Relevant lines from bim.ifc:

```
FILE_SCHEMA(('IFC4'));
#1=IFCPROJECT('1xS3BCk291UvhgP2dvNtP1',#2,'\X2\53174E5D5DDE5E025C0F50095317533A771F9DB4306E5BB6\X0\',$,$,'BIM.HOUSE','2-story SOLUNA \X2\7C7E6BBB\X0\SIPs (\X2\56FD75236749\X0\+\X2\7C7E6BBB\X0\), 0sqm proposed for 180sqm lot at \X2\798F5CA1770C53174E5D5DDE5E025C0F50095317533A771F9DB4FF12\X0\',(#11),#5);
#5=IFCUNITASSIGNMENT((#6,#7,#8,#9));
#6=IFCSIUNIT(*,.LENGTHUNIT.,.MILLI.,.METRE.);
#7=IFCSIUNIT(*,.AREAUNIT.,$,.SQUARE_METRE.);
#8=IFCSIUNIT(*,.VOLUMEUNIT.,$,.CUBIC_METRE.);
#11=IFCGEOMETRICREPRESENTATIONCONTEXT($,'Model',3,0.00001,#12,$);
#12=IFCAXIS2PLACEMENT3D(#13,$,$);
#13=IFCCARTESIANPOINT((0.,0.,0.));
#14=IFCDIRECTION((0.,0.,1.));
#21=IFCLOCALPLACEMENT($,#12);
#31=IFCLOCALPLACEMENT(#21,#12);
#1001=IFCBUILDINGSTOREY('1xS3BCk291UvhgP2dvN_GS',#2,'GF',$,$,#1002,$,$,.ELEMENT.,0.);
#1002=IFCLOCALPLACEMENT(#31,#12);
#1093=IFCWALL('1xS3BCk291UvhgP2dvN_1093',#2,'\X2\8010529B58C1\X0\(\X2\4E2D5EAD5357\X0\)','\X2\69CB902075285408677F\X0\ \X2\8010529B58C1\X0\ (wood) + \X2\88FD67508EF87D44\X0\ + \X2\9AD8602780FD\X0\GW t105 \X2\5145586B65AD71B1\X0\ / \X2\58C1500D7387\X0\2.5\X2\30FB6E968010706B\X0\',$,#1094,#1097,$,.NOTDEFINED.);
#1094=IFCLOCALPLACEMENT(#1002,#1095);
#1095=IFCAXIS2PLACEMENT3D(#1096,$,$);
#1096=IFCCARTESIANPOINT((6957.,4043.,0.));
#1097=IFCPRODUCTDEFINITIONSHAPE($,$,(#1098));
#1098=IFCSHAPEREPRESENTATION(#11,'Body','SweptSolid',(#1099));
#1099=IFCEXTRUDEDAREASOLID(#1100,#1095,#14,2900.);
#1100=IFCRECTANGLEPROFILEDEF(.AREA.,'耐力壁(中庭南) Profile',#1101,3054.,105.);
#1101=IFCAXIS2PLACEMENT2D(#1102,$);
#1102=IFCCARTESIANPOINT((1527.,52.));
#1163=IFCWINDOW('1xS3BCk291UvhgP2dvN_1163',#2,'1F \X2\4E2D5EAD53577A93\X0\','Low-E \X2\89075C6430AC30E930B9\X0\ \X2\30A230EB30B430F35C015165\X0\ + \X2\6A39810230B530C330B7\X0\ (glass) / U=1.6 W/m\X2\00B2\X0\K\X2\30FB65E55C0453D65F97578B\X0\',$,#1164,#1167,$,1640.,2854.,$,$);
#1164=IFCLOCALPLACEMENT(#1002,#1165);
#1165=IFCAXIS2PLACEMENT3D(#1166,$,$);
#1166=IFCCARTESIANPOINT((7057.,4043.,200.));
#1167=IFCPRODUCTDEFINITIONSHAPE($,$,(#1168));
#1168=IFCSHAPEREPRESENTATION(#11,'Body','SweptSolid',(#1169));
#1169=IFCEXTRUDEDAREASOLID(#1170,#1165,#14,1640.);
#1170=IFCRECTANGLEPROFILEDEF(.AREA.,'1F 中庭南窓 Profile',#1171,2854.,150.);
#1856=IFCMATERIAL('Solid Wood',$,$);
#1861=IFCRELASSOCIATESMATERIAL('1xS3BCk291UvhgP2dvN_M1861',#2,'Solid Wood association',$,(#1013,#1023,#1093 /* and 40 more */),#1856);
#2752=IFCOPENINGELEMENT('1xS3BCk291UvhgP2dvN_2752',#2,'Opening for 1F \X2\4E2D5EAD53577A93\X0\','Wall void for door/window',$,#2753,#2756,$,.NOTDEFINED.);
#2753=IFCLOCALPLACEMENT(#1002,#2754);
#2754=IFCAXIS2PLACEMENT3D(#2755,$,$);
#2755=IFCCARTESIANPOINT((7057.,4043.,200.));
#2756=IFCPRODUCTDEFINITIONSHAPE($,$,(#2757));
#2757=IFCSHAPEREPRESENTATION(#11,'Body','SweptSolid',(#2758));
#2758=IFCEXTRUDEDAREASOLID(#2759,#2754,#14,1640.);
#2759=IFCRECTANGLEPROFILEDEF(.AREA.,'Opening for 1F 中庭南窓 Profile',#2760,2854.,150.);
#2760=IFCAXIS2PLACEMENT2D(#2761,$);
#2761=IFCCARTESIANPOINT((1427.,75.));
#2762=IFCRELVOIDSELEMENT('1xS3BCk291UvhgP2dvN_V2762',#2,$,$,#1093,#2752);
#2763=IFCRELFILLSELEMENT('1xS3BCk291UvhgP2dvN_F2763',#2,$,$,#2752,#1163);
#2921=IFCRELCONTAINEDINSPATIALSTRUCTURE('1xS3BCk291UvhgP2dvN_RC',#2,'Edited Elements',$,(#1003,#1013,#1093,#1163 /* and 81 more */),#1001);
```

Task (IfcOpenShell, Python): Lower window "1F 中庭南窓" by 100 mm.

```python
import numpy as np
import ifcopenshell
import ifcopenshell.api.geometry
import ifcopenshell.util.placement
import ifcopenshell.util.unit

model = ifcopenshell.open("bim.ifc")
unit_scale = ifcopenshell.util.unit.calculate_unit_scale(model)

window = model.by_guid("1xS3BCk291UvhgP2dvN_1163")
opening = window.FillsVoids[0].RelatingOpeningElement
dz = -100.0

shift = np.array([0.0, 0.0, dz])
# The window is not placed relative to its opening, so move both.
for product in (opening, window):
    matrix = ifcopenshell.util.placement.get_local_placement(product.ObjectPlacement)
    matrix[:3, 3] += shift
    ifcopenshell.api.geometry.edit_object_placement(model, product=product, matrix=matrix, is_si=False)

print(f"moved by {dz * unit_scale:+.3f} m")

model.write("bim_rev.ifc")
```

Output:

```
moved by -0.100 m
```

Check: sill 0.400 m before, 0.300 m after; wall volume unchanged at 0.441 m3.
